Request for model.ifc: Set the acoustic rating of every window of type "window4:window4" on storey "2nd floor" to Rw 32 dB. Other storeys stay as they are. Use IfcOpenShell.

First a look at what the model holds.

```python
import ifcopenshell
import ifcopenshell.util.element

model = ifcopenshell.open("model.ifc")
print(model.schema)
storey = next(s for s in model.by_type("IfcBuildingStorey") if s.Name == "2nd floor")
windows = [e for e in ifcopenshell.util.element.get_decomposition(storey) if e.is_a("IfcWindow")]
seen = {}
for e in windows:
    element_type = ifcopenshell.util.element.get_type(e)
    key = (element_type.Name if element_type != e and element_type else None, ifcopenshell.util.element.get_pset(e, "Pset_WindowCommon", "AcousticRating"))
    seen[key] = seen.get(key, 0) + 1
for (name, value), count in sorted(seen.items(), key=str):
    print(count, "x", name, "|", value)
```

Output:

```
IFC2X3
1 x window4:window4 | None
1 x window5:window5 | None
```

```python
import ifcopenshell
import ifcopenshell.api.pset
import ifcopenshell.util.element

model = ifcopenshell.open("model.ifc")

storey = next(s for s in model.by_type("IfcBuildingStorey") if s.Name == "2nd floor")
windows = [e for e in ifcopenshell.util.element.get_decomposition(storey) if e.is_a("IfcWindow")]

count = 0
for e in windows:
    element_type = ifcopenshell.util.element.get_type(e)
    if element_type in (None, e) or element_type.Name != "window4:window4":
        continue
    # add_pset returns the element's existing set when there is one.
    pset = ifcopenshell.api.pset.add_pset(model, product=e, name="Pset_WindowCommon")
    ifcopenshell.api.pset.edit_pset(model, pset=pset, properties={"AcousticRating": "Rw 32 dB"})
    count += 1

print(count, "windows updated")

model.write("model_rev.ifc")
```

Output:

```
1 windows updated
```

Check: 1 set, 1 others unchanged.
